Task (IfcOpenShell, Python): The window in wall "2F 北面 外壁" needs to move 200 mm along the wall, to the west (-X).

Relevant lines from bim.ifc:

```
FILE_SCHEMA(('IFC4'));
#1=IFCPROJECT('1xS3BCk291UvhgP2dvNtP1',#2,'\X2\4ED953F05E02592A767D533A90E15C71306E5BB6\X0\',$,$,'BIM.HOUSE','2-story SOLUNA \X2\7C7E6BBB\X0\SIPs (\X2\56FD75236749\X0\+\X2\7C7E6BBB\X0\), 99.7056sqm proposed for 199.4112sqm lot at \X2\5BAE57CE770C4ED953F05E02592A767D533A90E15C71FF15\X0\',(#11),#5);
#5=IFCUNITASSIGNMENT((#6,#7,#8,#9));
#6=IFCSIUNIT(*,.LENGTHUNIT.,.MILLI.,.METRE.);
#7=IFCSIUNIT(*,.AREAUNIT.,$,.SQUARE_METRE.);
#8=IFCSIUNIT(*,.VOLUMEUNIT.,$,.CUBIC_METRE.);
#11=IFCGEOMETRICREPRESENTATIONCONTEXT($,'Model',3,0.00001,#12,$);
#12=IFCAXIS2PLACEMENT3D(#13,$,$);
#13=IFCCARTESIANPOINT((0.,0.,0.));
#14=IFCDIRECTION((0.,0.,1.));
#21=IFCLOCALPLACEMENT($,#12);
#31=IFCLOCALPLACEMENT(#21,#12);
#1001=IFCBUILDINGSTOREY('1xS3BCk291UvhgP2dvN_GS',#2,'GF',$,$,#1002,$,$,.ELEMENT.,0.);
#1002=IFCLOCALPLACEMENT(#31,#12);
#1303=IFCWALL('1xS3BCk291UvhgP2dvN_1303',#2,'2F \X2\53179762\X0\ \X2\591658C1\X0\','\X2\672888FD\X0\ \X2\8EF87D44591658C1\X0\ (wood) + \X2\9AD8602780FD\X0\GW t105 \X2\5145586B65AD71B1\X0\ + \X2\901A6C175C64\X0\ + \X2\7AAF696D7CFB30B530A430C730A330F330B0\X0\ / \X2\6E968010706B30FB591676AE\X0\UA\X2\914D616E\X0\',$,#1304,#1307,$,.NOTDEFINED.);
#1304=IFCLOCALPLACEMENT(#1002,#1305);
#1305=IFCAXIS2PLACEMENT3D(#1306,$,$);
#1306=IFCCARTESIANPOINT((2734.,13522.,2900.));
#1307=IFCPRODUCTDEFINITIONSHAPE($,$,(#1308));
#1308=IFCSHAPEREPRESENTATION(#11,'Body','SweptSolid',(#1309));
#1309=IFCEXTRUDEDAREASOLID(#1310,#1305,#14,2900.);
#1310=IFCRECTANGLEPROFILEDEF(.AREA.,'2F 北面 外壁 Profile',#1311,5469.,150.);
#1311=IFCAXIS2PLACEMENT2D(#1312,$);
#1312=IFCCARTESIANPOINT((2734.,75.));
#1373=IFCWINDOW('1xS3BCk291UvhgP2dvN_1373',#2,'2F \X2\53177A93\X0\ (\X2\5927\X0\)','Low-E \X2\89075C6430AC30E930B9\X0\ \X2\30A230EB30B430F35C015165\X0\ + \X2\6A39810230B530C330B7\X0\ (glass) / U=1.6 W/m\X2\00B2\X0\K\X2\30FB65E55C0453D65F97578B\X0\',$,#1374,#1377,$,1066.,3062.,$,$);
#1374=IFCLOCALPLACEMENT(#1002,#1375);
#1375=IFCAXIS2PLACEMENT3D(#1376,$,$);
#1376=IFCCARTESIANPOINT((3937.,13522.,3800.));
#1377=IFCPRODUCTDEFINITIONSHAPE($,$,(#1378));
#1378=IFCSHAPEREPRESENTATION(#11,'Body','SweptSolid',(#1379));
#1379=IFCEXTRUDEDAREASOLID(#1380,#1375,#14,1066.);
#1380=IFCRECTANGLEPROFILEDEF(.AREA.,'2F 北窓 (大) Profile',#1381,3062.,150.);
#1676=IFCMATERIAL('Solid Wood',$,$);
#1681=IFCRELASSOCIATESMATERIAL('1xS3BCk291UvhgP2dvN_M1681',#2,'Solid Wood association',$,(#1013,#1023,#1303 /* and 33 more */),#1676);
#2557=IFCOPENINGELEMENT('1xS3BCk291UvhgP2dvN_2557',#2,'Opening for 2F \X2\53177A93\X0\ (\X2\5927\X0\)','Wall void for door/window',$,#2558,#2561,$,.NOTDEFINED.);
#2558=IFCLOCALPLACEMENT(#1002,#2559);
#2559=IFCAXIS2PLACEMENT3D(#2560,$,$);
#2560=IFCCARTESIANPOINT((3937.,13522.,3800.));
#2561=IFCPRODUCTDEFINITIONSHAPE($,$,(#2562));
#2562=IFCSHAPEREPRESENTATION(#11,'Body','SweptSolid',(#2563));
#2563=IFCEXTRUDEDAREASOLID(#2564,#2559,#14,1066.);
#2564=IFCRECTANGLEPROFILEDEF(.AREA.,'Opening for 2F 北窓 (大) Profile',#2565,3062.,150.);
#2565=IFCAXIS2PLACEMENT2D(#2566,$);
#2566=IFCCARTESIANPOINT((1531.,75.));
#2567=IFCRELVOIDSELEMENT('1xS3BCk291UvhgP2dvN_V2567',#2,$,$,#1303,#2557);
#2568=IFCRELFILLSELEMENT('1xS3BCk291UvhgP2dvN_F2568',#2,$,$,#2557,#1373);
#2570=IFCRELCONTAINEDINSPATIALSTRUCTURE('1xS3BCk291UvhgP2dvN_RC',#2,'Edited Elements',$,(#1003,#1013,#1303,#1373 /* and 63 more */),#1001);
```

```python
import ifcopenshell
import ifcopenshell.api.geometry
import ifcopenshell.util.placement

model = ifcopenshell.open("bim.ifc")

window = model.by_guid("1xS3BCk291UvhgP2dvN_1373")
opening = window.FillsVoids[0].RelatingOpeningElement
wall = opening.VoidsElements[0].RelatingBuildingElement

wall_matrix = ifcopenshell.util.placement.get_local_placement(wall.ObjectPlacement)
shift = wall_matrix[:3, 0] * -200.0
before = ifcopenshell.util.placement.get_local_placement(window.ObjectPlacement)[:3, 3].copy()

# The window is not placed relative to its opening, so move both.
for product in (opening, window):
    matrix = ifcopenshell.util.placement.get_local_placement(product.ObjectPlacement)
    matrix[:3, 3] += shift
    ifcopenshell.api.geometry.edit_object_placement(model, product=product, matrix=matrix, is_si=False)

after = ifcopenshell.util.placement.get_local_placement(window.ObjectPlacement)[:3, 3]
print("window moved by", (after - before).round(3) + 0.0)

model.write("bim_updated.ifc")
```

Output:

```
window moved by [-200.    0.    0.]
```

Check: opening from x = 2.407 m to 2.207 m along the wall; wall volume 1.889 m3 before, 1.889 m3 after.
